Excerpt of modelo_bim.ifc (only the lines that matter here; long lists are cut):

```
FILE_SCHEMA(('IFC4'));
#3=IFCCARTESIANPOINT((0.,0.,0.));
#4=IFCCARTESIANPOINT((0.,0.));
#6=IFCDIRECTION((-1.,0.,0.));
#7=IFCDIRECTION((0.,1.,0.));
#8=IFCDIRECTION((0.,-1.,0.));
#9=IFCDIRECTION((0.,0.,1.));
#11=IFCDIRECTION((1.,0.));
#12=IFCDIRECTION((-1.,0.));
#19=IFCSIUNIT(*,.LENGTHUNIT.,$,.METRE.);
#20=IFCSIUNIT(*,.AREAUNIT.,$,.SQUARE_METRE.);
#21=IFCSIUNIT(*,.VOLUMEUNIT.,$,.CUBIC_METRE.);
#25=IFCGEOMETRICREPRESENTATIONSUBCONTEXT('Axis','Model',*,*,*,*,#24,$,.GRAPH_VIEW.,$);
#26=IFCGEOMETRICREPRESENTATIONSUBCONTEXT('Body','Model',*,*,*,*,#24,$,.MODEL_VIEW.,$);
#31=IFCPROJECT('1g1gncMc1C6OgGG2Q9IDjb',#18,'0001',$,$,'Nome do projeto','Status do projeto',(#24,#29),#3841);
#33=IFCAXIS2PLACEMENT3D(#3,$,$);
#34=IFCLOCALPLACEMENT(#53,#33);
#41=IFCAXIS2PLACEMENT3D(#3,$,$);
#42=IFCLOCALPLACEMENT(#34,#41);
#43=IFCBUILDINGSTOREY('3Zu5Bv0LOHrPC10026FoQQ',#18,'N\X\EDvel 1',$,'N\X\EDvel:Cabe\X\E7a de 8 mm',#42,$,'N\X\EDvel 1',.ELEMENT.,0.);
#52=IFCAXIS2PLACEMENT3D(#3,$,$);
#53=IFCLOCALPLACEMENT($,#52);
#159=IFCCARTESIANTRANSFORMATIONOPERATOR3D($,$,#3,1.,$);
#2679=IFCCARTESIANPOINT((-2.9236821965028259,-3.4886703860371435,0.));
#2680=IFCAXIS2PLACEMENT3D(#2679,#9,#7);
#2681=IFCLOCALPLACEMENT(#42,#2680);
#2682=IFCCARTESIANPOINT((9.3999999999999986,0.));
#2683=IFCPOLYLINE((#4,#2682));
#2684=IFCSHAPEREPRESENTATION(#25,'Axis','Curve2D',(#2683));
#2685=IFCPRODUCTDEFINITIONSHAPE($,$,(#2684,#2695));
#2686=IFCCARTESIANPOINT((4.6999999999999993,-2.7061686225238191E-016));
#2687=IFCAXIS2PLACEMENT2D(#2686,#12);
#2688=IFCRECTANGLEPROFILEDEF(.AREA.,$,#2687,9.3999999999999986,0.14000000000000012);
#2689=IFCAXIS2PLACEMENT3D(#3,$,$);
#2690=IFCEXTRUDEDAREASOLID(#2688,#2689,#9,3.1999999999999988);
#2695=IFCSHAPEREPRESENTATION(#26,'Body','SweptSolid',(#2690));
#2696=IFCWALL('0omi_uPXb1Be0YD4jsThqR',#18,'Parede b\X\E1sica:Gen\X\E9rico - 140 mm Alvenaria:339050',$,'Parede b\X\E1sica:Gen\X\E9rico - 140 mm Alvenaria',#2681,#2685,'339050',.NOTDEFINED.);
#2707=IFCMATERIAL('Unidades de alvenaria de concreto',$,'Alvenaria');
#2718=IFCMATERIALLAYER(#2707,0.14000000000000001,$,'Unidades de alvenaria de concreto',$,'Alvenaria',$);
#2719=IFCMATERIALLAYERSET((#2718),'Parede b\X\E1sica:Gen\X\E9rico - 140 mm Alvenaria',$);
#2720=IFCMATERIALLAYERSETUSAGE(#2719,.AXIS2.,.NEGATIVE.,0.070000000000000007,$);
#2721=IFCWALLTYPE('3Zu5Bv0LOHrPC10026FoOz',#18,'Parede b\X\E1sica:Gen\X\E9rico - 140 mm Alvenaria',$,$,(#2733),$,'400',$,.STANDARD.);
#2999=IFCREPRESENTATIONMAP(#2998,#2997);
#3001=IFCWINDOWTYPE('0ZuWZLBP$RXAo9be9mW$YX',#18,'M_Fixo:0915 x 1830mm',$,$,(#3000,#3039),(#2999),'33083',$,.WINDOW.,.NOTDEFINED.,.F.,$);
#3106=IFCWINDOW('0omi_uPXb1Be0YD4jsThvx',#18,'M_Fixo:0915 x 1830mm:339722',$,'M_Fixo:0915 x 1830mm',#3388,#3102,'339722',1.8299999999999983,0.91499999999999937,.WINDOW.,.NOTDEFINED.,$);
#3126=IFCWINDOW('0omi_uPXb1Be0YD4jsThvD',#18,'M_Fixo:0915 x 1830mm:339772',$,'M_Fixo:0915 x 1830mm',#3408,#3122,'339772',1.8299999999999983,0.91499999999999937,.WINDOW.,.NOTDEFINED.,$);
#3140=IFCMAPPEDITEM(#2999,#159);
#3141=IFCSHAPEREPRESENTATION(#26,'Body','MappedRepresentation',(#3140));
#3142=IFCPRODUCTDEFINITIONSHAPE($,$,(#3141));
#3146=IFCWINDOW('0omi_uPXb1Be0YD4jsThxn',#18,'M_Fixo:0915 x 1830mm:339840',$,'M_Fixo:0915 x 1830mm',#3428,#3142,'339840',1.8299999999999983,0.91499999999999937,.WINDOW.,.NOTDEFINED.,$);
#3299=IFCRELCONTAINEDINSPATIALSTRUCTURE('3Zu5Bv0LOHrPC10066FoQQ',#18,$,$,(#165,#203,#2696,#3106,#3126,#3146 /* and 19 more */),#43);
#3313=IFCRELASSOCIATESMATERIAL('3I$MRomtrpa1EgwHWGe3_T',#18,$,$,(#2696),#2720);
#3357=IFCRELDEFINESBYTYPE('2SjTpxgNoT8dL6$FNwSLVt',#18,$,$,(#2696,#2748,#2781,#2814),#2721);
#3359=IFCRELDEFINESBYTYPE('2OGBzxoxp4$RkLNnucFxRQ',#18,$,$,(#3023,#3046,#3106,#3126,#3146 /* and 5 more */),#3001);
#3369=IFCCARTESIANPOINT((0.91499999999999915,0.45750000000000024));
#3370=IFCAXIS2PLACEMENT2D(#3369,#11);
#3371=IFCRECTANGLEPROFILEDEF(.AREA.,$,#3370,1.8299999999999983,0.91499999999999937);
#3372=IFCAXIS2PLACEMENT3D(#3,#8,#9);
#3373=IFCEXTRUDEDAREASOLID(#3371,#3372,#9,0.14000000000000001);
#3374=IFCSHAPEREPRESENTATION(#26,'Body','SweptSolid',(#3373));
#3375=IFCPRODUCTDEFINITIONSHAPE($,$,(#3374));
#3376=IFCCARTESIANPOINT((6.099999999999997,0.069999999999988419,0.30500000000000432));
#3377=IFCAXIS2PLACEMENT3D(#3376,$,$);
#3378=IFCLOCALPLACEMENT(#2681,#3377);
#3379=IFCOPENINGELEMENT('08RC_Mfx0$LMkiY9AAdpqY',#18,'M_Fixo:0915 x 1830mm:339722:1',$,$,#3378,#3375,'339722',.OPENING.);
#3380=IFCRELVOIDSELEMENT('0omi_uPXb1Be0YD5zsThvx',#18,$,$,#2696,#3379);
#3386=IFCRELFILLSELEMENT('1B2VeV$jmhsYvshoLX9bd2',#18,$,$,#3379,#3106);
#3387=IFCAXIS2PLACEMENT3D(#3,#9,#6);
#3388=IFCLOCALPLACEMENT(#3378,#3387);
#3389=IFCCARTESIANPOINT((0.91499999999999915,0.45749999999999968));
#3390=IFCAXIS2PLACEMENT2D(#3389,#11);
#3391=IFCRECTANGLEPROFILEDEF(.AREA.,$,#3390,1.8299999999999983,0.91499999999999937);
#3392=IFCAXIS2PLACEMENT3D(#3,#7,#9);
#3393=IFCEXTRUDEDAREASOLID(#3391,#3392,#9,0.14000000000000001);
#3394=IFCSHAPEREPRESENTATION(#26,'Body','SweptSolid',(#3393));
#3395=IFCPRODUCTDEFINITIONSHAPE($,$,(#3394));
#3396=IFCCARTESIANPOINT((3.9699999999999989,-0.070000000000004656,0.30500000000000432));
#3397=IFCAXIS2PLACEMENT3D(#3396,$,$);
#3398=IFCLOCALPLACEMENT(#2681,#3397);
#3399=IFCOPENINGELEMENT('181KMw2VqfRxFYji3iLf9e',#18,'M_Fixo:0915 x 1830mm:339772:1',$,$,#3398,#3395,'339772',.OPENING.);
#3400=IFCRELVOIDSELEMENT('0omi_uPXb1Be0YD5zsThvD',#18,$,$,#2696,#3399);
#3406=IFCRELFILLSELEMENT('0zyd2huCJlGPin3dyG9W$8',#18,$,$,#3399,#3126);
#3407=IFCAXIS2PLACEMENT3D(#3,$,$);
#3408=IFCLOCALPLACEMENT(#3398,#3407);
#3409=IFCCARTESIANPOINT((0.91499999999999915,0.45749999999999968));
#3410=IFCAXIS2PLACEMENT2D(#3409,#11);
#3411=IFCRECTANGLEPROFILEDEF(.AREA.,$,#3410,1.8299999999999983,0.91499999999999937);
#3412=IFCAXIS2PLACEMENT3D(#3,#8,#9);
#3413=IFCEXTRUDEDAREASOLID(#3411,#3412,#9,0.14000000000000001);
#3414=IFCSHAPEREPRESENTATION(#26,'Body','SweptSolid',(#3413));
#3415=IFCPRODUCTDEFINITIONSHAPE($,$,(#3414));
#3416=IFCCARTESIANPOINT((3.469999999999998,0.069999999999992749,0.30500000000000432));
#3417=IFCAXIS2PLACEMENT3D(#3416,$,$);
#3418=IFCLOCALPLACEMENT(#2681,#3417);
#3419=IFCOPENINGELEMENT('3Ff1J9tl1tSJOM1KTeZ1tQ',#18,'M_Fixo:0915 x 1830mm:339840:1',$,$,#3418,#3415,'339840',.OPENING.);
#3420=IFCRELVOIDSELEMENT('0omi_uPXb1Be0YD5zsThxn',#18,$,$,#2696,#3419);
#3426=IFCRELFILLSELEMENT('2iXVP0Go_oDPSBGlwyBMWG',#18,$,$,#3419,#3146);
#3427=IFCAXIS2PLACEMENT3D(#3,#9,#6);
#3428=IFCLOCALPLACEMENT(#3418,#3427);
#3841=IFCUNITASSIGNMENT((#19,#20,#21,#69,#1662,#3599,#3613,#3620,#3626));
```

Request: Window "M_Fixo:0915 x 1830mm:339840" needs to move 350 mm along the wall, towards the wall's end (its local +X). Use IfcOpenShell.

```python
import ifcopenshell
import ifcopenshell.api.geometry
import ifcopenshell.util.placement
import ifcopenshell.util.unit

model = ifcopenshell.open("modelo_bim.ifc")
unit_scale = ifcopenshell.util.unit.calculate_unit_scale(model)

window = model.by_guid("0omi_uPXb1Be0YD4jsThxn")
opening = window.FillsVoids[0].RelatingOpeningElement
wall = opening.VoidsElements[0].RelatingBuildingElement

wall_matrix = ifcopenshell.util.placement.get_local_placement(wall.ObjectPlacement)
shift = wall_matrix[:3, 0] * 0.35 / unit_scale
before = ifcopenshell.util.placement.get_local_placement(window.ObjectPlacement)[:3, 3].copy()

# The window is placed relative to its opening, so it follows when the opening moves.
matrix = ifcopenshell.util.placement.get_local_placement(opening.ObjectPlacement)
matrix[:3, 3] += shift
ifcopenshell.api.geometry.edit_object_placement(
    model, product=opening, matrix=matrix, is_si=False, should_transform_children=True
)

after = ifcopenshell.util.placement.get_local_placement(window.ObjectPlacement)[:3, 3]
print("window moved by", (after - before).round(3) + 0.0)

model.write("modelo_bim_updated.ifc")
```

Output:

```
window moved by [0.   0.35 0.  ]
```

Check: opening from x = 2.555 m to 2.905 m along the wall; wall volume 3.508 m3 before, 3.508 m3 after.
